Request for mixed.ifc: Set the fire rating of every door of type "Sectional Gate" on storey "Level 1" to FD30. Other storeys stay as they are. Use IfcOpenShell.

First a look at what the model holds.

```python
import ifcopenshell
import ifcopenshell.util.element

model = ifcopenshell.open("mixed.ifc")
print(model.schema)
storey = next(s for s in model.by_type("IfcBuildingStorey") if s.Name == "Level 1")
doors = [e for e in ifcopenshell.util.element.get_decomposition(storey) if e.is_a("IfcDoor")]
seen = {}
for e in doors:
    element_type = ifcopenshell.util.element.get_type(e)
    key = (element_type.Name if element_type != e and element_type else None, ifcopenshell.util.element.get_pset(e, "Pset_DoorCommon", "FireRating"))
    seen[key] = seen.get(key, 0) + 1
for (name, value), count in sorted(seen.items(), key=str):
    print(count, "x", name, "|", value)
```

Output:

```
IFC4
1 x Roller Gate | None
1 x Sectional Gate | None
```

```python
import ifcopenshell
import ifcopenshell.api.pset
import ifcopenshell.util.element

model = ifcopenshell.open("mixed.ifc")

storey = next(s for s in model.by_type("IfcBuildingStorey") if s.Name == "Level 1")
doors = [e for e in ifcopenshell.util.element.get_decomposition(storey) if e.is_a("IfcDoor")]

count = 0
for e in doors:
    element_type = ifcopenshell.util.element.get_type(e)
    if element_type in (None, e) or element_type.Name != "Sectional Gate":
        continue
    # add_pset returns the element's existing set when there is one.
    pset = ifcopenshell.api.pset.add_pset(model, product=e, name="Pset_DoorCommon")
    ifcopenshell.api.pset.edit_pset(model, pset=pset, properties={"FireRating": "FD30"})
    count += 1

print(count, "doors updated")

model.write("mixed_updated.ifc")
```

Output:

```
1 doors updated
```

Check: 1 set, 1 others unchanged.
